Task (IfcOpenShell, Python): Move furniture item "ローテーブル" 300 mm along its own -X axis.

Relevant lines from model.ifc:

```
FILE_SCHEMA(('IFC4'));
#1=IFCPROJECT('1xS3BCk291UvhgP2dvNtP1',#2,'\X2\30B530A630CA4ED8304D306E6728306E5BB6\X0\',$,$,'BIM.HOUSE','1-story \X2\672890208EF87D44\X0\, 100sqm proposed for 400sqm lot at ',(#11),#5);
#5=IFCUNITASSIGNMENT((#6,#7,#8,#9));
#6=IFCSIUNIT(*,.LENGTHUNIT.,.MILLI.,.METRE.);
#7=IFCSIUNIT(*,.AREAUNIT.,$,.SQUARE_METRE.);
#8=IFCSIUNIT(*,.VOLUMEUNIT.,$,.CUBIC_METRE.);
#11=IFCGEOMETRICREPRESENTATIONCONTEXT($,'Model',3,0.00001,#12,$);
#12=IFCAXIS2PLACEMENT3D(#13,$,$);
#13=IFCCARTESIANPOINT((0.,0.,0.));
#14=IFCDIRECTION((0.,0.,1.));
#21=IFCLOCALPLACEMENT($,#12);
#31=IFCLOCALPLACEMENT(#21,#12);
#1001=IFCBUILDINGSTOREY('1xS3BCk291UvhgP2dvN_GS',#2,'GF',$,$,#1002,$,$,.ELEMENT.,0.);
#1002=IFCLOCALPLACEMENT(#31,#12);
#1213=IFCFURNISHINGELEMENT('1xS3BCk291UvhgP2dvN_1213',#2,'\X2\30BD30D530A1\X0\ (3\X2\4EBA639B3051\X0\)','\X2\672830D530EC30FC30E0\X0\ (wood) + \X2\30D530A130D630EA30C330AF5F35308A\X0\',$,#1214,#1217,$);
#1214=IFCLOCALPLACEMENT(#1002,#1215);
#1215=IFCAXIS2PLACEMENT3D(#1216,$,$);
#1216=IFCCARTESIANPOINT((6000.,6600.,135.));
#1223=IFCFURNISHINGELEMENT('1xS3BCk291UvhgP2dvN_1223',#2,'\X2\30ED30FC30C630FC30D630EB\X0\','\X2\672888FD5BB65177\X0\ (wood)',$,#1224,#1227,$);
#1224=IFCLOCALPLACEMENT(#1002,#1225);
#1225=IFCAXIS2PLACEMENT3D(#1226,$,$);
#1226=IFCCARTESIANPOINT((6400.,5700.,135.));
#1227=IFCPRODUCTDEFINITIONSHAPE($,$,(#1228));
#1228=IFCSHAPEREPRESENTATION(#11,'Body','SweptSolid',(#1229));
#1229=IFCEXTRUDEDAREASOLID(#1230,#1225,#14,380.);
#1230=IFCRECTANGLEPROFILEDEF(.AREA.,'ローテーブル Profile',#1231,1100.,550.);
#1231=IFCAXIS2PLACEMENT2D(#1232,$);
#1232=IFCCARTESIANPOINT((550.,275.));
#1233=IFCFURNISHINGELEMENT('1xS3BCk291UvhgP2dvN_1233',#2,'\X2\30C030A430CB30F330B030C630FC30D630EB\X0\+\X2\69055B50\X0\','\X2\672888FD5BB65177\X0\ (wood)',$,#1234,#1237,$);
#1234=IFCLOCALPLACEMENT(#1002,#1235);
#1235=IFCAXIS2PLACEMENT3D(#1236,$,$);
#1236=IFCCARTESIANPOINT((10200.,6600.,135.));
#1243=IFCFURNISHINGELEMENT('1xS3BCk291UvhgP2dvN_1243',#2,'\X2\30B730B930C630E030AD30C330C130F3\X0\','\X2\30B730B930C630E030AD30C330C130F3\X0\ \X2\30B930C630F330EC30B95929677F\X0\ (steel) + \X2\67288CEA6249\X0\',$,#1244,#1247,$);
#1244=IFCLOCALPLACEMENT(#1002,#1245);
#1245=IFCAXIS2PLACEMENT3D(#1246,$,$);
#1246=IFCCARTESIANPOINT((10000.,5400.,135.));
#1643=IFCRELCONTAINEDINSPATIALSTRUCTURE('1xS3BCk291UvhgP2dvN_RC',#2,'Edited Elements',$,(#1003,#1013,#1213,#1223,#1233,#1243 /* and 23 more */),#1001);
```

```python
import ifcopenshell
import ifcopenshell.api.geometry
import ifcopenshell.util.placement
import ifcopenshell.util.unit

model = ifcopenshell.open("model.ifc")
unit_scale = ifcopenshell.util.unit.calculate_unit_scale(model)

item = model.by_guid("1xS3BCk291UvhgP2dvN_1223")
matrix = ifcopenshell.util.placement.get_local_placement(item.ObjectPlacement)
matrix[:3, 3] -= matrix[:3, 0] * 0.3 / unit_scale
ifcopenshell.api.geometry.edit_object_placement(model, product=item, matrix=matrix, is_si=False)

print(ifcopenshell.util.placement.get_local_placement(item.ObjectPlacement).round(3) + 0.0)

model.write("model_rev.ifc")
```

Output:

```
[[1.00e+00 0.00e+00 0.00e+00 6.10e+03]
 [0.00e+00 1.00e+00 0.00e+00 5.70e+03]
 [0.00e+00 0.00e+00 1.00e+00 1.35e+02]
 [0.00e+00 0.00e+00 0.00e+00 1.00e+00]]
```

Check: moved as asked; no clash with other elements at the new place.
